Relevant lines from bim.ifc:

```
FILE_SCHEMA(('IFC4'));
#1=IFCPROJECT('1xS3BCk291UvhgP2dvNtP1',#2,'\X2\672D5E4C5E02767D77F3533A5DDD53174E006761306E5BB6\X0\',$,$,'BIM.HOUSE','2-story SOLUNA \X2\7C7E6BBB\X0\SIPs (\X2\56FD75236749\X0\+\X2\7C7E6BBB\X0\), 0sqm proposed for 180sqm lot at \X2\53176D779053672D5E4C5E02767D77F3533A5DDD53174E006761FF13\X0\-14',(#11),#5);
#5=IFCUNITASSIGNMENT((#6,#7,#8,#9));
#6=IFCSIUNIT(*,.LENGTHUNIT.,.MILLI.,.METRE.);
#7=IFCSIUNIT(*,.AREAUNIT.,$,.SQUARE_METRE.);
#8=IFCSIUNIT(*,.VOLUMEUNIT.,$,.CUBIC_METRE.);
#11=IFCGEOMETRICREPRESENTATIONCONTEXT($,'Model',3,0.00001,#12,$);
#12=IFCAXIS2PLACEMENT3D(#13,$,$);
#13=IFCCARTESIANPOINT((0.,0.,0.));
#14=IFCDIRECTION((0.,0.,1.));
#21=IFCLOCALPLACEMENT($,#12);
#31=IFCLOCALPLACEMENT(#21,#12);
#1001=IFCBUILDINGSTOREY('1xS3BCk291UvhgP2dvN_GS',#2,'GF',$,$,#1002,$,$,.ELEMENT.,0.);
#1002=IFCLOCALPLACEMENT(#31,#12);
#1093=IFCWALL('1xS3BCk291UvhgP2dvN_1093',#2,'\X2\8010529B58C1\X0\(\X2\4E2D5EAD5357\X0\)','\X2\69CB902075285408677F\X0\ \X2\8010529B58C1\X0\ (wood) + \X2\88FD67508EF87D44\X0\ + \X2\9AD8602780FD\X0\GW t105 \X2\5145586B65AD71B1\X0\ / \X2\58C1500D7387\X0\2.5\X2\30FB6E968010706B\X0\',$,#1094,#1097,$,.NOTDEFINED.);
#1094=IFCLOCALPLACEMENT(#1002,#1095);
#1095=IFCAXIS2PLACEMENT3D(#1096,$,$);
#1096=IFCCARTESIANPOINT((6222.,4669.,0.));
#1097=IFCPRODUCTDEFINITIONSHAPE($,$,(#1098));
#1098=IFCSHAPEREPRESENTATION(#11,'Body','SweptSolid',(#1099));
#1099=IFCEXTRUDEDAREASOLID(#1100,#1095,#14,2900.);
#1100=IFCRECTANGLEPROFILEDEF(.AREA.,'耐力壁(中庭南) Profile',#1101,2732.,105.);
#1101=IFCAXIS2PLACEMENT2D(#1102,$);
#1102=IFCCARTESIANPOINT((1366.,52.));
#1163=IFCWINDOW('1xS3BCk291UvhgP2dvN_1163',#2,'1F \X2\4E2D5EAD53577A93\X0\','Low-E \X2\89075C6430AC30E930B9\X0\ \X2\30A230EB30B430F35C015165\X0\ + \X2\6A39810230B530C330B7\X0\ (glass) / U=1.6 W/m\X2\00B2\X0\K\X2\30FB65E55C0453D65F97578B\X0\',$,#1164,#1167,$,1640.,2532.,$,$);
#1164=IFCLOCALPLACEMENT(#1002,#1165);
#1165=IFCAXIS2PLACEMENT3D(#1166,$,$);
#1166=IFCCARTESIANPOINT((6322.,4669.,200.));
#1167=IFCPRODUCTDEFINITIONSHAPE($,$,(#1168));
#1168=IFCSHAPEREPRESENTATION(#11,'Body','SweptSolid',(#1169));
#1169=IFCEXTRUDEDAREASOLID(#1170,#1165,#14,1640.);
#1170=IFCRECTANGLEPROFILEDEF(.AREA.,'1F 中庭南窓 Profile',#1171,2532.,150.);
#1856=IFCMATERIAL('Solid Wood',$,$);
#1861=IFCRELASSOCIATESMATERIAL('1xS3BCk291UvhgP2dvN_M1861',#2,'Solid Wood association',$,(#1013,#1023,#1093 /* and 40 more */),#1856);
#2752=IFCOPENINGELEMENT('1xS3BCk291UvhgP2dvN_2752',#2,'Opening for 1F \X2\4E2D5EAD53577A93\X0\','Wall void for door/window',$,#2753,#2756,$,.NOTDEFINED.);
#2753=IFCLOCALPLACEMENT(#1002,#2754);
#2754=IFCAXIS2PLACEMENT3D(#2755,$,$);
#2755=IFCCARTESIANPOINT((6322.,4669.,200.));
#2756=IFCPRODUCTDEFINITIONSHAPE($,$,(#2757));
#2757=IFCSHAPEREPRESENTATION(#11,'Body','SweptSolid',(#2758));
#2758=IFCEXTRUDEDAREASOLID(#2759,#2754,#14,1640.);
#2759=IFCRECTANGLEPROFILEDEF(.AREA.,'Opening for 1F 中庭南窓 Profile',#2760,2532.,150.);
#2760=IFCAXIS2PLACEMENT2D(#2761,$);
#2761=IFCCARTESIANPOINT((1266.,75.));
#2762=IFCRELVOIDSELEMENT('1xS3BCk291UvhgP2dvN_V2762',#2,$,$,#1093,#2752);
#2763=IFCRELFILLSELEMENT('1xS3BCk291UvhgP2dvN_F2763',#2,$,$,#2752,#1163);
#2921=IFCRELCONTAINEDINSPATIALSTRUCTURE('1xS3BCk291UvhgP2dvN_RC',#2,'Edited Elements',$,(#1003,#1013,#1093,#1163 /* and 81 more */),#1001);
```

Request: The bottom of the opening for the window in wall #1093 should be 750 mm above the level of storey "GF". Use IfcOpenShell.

```python
import numpy as np
import ifcopenshell
import ifcopenshell.api.geometry
import ifcopenshell.geom
import ifcopenshell.util.element
import ifcopenshell.util.placement
import ifcopenshell.util.shape
import ifcopenshell.util.unit

model = ifcopenshell.open("bim.ifc")
unit_scale = ifcopenshell.util.unit.calculate_unit_scale(model)

window = model.by_id(1163)
opening = window.FillsVoids[0].RelatingOpeningElement
storey = ifcopenshell.util.element.get_container(window, ifc_class="IfcBuildingStorey")
level = ifcopenshell.util.placement.get_local_placement(storey.ObjectPlacement)[2, 3]

# The opening's origin need not be at the sill, so measure its lowest point.
shape = ifcopenshell.geom.create_shape(ifcopenshell.geom.settings(), opening)
bottom = ifcopenshell.util.shape.get_shape_bottom_elevation(shape, shape.geometry) / unit_scale
dz = level + 0.75 / unit_scale - bottom

shift = np.array([0.0, 0.0, dz])
# The window is not placed relative to its opening, so move both.
for product in (opening, window):
    matrix = ifcopenshell.util.placement.get_local_placement(product.ObjectPlacement)
    matrix[:3, 3] += shift
    ifcopenshell.api.geometry.edit_object_placement(model, product=product, matrix=matrix, is_si=False)

print(f"moved by {dz * unit_scale:+.3f} m")

model.write("bim_edited.ifc")
```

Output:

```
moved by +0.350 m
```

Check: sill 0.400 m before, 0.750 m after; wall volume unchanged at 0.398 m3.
